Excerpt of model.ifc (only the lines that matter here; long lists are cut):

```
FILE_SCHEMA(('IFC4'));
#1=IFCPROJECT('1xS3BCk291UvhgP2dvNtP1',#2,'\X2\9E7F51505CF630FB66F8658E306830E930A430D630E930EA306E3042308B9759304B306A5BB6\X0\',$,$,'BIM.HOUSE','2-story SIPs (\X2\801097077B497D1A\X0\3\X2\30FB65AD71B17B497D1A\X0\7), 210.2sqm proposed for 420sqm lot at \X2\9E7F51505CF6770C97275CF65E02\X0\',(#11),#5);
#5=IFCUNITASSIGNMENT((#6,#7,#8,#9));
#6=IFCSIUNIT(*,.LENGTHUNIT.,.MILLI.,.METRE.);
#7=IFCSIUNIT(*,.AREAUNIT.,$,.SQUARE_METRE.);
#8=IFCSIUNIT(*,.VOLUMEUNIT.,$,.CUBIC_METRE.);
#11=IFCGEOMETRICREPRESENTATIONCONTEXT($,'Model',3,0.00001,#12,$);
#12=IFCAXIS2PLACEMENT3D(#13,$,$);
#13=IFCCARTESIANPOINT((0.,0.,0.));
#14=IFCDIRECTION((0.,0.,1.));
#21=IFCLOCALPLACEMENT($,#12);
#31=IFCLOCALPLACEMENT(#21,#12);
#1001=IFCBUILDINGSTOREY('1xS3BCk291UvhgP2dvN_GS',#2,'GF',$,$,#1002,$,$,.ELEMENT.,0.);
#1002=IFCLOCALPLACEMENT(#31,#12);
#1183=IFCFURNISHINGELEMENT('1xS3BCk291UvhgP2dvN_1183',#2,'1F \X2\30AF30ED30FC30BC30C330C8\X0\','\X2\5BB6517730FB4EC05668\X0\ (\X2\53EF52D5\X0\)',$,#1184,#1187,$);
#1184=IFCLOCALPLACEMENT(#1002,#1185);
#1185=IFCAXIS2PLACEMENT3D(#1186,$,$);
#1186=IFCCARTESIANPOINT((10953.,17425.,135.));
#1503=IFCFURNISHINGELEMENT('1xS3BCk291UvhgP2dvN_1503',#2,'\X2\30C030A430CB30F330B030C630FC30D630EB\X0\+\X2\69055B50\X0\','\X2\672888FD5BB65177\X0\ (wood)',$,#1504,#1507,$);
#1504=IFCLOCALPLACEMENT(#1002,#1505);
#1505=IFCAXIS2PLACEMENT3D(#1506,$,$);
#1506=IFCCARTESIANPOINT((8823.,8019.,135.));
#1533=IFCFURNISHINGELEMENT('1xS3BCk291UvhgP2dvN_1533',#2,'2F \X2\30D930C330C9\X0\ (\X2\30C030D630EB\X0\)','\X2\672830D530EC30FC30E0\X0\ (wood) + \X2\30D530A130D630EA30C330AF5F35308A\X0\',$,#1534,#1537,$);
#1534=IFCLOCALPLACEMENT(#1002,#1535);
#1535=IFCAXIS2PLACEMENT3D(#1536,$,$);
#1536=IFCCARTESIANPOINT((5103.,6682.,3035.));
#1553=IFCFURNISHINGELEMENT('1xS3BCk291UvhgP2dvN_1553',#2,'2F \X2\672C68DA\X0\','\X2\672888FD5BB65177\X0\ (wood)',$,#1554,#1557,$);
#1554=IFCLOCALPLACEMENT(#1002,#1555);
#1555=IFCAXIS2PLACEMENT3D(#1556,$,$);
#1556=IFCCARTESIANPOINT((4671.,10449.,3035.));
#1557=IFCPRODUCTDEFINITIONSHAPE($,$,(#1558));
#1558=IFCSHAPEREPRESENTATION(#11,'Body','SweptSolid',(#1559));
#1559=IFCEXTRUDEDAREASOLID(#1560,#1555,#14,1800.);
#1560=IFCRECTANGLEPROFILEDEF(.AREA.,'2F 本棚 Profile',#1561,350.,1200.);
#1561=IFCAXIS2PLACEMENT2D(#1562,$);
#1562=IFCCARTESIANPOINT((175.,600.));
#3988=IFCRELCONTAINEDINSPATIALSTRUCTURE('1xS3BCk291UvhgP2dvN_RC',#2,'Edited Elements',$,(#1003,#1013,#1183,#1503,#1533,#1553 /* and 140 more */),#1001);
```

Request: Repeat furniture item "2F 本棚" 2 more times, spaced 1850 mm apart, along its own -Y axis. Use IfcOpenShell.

```python
import ifcopenshell
import ifcopenshell.api.geometry
import ifcopenshell.api.root
import ifcopenshell.util.element
import ifcopenshell.util.placement
import ifcopenshell.util.unit

model = ifcopenshell.open("model.ifc")
unit_scale = ifcopenshell.util.unit.calculate_unit_scale(model)


def reuse_history(source, copy):
    """copy_class also copies each property set's owner history, people and application; keep the originals."""
    for rel in copy.IsDefinedBy:
        if rel.is_a("IfcRelDefinesByProperties") and (history := rel.RelatingPropertyDefinition.OwnerHistory):
            rel.RelatingPropertyDefinition.OwnerHistory = source.OwnerHistory
            ifcopenshell.util.element.remove_deep2(model, history)


source = model.by_id(1553)
base = ifcopenshell.util.placement.get_local_placement(source.ObjectPlacement)
step = -base[:3, 1] * 1.85 / unit_scale

for i in range(1, 3):
    copy = ifcopenshell.api.root.copy_class(model, product=source)
    copy.Representation = ifcopenshell.util.element.copy_deep(
        model, source.Representation, exclude=["IfcGeometricRepresentationContext", "IfcRepresentationMap"]
    )
    reuse_history(source, copy)
    matrix = base.copy()
    matrix[:3, 3] += i * step
    print("added at", matrix[:3, 3].round(3) + 0.0)
    ifcopenshell.api.geometry.edit_object_placement(model, product=copy, matrix=matrix, is_si=False)

model.write("model_edited.ifc")
```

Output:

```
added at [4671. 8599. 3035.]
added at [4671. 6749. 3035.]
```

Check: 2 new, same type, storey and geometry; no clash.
